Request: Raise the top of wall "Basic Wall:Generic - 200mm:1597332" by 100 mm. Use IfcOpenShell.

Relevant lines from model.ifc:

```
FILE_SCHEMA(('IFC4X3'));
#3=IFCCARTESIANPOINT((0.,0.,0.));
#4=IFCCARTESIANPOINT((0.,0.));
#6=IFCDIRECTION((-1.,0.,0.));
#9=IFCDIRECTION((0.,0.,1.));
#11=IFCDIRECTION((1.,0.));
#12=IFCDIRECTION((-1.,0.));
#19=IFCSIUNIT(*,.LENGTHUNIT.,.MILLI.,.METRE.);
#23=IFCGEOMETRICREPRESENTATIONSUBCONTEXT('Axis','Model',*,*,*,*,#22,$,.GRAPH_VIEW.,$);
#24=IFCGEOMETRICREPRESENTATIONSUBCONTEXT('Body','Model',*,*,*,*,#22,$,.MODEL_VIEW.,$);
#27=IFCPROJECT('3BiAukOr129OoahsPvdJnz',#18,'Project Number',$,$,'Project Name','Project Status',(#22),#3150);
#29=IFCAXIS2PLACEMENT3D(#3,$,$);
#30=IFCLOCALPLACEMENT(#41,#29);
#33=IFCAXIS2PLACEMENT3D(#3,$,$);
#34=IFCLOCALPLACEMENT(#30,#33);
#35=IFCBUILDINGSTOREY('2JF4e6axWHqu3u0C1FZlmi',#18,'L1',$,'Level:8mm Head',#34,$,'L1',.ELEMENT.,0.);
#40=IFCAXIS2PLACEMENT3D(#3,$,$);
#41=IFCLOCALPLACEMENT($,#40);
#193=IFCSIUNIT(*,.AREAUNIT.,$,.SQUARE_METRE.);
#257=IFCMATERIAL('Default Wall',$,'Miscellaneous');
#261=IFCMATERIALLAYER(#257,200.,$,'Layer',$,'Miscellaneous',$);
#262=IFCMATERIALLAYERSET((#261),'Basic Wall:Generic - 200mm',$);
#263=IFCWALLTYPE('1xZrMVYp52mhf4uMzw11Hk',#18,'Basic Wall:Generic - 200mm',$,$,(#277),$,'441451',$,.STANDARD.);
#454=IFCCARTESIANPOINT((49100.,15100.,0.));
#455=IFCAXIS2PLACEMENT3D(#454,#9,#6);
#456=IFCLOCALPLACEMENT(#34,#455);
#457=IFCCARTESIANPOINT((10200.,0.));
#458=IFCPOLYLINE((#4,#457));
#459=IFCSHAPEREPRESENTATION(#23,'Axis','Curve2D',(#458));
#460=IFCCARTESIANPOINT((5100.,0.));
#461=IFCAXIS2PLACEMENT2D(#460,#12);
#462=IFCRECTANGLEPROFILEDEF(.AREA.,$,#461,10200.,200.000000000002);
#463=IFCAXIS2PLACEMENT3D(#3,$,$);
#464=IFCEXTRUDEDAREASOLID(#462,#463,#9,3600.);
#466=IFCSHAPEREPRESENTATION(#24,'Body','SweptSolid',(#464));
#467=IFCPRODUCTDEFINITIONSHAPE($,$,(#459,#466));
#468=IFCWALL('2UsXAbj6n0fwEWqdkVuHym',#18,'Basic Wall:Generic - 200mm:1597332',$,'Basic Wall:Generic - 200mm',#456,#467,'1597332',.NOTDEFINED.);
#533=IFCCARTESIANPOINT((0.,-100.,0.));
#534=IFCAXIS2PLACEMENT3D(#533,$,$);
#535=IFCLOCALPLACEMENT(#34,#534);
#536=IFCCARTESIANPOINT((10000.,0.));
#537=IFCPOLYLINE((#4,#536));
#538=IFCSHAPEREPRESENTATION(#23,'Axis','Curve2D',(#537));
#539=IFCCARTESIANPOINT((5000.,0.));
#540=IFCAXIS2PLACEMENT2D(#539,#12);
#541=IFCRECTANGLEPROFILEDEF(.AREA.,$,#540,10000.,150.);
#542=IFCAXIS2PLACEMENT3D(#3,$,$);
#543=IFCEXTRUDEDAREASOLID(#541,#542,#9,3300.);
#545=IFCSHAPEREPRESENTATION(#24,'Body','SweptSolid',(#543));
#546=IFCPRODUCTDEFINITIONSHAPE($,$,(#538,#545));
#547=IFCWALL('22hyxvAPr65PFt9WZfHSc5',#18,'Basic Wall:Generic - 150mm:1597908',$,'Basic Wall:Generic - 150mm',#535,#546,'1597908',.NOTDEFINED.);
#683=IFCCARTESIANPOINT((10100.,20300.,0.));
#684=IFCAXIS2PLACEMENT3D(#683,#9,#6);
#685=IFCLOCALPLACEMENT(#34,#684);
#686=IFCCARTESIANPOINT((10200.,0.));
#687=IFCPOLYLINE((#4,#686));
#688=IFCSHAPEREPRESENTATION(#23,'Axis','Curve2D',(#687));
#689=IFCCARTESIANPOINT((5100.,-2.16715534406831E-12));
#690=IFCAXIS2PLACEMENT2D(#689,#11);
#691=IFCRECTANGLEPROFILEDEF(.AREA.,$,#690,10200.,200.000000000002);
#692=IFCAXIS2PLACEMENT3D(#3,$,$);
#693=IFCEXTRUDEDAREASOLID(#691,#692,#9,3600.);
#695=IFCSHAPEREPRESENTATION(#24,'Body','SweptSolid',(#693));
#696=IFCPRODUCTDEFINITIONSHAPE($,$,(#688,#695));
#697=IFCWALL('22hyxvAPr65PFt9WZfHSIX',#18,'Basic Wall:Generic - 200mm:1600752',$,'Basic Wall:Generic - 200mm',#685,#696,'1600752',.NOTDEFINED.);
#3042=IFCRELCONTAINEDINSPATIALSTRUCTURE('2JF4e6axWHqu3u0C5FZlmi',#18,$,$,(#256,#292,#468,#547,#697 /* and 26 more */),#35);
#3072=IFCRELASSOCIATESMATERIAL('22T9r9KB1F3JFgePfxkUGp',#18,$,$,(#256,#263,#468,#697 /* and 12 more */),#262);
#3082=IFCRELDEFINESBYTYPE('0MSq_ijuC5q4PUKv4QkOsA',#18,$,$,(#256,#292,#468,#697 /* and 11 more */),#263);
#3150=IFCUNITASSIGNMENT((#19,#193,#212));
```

```python
import ifcopenshell
import ifcopenshell.geom
import ifcopenshell.util.representation
import ifcopenshell.util.shape
import ifcopenshell.util.unit

model = ifcopenshell.open("model.ifc")
unit_scale = ifcopenshell.util.unit.calculate_unit_scale(model)
settings = ifcopenshell.geom.settings()


def volume(element):
    """Net volume in cubic metres, openings subtracted."""
    shape = ifcopenshell.geom.create_shape(settings, element)
    return ifcopenshell.util.shape.get_volume(shape.geometry)


wall = model.by_guid("2UsXAbj6n0fwEWqdkVuHym")
before = volume(wall)

body = ifcopenshell.util.representation.get_representation(wall, "Model", "Body")
solid = body.Items[0]
old_height = solid.Depth
solid.Depth += 0.1 / unit_scale
after = volume(wall)

print(f"height {old_height:g} -> {solid.Depth:g}, volume {before:.3f} -> {after:.3f} m3")

model.write("model-out.ifc")
```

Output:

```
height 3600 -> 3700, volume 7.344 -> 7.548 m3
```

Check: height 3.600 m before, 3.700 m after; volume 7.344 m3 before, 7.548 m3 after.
